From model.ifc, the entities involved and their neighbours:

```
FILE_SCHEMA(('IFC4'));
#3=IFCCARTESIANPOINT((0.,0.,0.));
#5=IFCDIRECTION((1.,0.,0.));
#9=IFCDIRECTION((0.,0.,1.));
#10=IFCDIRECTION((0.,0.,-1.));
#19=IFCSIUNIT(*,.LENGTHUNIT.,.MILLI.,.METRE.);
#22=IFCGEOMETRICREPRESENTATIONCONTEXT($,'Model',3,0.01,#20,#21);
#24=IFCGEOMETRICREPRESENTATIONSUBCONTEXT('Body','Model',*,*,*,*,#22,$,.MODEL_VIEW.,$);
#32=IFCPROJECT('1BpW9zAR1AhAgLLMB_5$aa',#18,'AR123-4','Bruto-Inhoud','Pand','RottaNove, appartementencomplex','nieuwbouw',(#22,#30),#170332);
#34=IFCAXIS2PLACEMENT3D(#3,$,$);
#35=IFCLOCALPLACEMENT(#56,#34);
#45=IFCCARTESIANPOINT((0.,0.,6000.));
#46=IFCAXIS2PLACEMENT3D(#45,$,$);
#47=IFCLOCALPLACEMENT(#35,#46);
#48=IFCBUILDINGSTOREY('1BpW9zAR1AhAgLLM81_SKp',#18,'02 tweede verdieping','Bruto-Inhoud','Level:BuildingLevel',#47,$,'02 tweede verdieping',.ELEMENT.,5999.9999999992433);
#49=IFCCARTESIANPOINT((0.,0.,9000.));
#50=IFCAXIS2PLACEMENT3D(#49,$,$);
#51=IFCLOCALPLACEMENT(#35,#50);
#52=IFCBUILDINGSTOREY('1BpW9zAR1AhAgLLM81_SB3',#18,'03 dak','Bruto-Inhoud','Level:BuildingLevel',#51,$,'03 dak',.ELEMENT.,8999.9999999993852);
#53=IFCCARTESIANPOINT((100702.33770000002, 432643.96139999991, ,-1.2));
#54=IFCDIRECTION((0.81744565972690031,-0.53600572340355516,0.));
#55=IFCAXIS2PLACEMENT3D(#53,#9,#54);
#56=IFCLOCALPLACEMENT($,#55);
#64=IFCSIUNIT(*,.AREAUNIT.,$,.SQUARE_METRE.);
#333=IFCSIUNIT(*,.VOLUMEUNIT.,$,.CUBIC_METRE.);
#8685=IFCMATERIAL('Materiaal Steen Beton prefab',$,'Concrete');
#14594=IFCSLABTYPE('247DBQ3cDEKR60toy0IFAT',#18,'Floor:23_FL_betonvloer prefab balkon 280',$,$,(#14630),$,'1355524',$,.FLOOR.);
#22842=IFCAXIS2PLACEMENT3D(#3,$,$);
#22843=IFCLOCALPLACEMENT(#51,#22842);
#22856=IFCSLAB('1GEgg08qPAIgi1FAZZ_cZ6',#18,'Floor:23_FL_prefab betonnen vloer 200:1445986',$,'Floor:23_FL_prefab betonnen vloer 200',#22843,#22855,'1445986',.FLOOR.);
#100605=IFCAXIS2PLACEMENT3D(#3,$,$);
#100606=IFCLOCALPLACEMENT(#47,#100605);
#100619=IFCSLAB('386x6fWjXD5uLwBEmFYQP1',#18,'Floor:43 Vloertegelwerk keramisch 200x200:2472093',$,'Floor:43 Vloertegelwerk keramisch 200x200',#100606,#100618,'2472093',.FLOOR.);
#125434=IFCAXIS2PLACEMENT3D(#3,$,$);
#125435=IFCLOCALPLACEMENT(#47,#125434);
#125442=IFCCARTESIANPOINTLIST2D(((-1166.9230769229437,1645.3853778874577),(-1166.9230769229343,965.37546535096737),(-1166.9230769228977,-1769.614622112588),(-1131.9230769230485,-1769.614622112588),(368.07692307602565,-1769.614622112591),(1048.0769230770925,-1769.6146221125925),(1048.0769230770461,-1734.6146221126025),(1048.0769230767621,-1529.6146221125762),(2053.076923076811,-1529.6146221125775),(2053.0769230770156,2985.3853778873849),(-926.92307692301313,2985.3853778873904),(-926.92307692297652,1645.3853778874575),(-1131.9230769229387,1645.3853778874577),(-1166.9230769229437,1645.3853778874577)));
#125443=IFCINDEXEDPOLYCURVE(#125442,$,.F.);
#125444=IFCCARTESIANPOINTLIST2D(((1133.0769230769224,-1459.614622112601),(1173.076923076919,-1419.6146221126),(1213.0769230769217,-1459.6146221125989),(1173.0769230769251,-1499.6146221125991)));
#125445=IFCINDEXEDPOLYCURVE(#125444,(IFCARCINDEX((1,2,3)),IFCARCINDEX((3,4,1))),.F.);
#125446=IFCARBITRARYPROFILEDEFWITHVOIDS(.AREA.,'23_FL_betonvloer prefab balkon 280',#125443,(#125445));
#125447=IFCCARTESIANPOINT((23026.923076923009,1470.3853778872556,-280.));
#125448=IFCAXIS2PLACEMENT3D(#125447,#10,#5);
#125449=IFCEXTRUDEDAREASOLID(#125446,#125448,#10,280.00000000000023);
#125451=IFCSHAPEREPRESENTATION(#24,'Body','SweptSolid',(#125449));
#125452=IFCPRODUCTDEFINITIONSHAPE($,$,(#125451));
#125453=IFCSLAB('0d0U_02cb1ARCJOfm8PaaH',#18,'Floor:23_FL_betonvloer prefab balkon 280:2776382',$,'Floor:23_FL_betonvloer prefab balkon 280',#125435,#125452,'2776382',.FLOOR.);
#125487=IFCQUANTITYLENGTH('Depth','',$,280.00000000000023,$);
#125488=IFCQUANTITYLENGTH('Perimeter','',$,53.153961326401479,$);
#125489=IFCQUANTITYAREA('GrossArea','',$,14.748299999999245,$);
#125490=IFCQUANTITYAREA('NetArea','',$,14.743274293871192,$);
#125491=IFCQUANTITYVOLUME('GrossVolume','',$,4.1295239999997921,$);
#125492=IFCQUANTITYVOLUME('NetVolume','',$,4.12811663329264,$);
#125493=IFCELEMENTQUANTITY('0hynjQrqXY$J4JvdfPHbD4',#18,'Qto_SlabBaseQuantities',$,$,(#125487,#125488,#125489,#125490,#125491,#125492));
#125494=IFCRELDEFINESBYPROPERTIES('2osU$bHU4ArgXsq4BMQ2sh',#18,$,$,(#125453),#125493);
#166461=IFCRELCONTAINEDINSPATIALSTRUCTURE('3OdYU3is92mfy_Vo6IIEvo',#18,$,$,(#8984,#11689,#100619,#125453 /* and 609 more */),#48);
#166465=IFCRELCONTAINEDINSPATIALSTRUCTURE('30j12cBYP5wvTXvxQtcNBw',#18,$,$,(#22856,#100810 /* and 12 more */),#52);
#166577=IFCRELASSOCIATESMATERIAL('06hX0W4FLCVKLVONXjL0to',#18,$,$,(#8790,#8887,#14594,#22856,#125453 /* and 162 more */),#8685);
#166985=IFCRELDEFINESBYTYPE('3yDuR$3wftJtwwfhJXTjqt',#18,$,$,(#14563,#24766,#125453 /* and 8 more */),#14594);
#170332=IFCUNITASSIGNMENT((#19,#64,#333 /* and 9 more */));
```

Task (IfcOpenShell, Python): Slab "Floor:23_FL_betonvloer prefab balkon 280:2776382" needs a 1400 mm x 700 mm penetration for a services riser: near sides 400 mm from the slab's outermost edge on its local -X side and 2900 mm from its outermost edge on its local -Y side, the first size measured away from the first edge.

```python
import numpy as np
import ifcopenshell
import ifcopenshell.api.feature
import ifcopenshell.api.geometry
import ifcopenshell.api.pset
import ifcopenshell.api.root
import ifcopenshell.geom
import ifcopenshell.util.element
import ifcopenshell.util.placement
import ifcopenshell.util.representation
import ifcopenshell.util.shape
import ifcopenshell.util.unit

model = ifcopenshell.open("model.ifc")
unit_scale = ifcopenshell.util.unit.calculate_unit_scale(model)
area_scale = ifcopenshell.util.unit.calculate_unit_scale(model, "AREAUNIT")
volume_scale = ifcopenshell.util.unit.calculate_unit_scale(model, "VOLUMEUNIT")
settings = ifcopenshell.geom.settings()


def volume(element):
    """Net volume in cubic metres, openings subtracted."""
    shape = ifcopenshell.geom.create_shape(settings, element)
    return ifcopenshell.util.shape.get_volume(shape.geometry)


slab = model.by_guid("0d0U_02cb1ARCJOfm8PaaH")
before = volume(slab)

# Extent in the slab's own axes, in metres. The edges named are its -X and -Y sides.
slab_shape = ifcopenshell.geom.create_shape(settings, slab)
vertices = ifcopenshell.util.shape.get_vertices(slab_shape.geometry)
x_min, y_min, bottom = vertices.min(axis=0)
top = vertices[:, 2].max()

opening = ifcopenshell.api.root.create_entity(model, ifc_class="IfcOpeningElement", name="Services riser opening", predefined_type="OPENING")
context = ifcopenshell.util.representation.get_context(model, "Model", "Body", "MODEL_VIEW")
width, depth = 1.4, 0.7
outline = [(0.0, 0.0), (width, 0.0), (width, depth), (0.0, depth), (0.0, 0.0)]
# Overshoot both faces by 50 mm so the cut is clean.
shape = ifcopenshell.api.geometry.add_slab_representation(
    model, context=context, depth=top - bottom + 0.1, polyline=outline
)
ifcopenshell.api.geometry.assign_representation(model, product=opening, representation=shape)

matrix = ifcopenshell.util.placement.get_local_placement(slab.ObjectPlacement)
matrix[:, 3] = matrix @ np.append(np.array([x_min + 0.4, y_min + 2.9, bottom - 0.05]) / unit_scale, 1.0)
ifcopenshell.api.geometry.edit_object_placement(model, product=opening, matrix=matrix, is_si=False)
ifcopenshell.api.feature.add_feature(model, feature=opening, element=slab)

after = volume(slab)

# Update the slab's stored quantities.
qto = model.by_id(ifcopenshell.util.element.get_pset(slab, "Qto_SlabBaseQuantities", should_inherit=False)["id"])
ifcopenshell.api.pset.edit_qto(model, qto=qto, properties={
    "NetArea": after / (top - bottom) / area_scale,
    "NetVolume": after / volume_scale,
})

print(f"slab volume {before:.3f} -> {after:.3f} m3")

model.write("model_v2.ifc")
```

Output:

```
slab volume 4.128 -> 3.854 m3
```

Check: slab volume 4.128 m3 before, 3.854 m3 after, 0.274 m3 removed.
